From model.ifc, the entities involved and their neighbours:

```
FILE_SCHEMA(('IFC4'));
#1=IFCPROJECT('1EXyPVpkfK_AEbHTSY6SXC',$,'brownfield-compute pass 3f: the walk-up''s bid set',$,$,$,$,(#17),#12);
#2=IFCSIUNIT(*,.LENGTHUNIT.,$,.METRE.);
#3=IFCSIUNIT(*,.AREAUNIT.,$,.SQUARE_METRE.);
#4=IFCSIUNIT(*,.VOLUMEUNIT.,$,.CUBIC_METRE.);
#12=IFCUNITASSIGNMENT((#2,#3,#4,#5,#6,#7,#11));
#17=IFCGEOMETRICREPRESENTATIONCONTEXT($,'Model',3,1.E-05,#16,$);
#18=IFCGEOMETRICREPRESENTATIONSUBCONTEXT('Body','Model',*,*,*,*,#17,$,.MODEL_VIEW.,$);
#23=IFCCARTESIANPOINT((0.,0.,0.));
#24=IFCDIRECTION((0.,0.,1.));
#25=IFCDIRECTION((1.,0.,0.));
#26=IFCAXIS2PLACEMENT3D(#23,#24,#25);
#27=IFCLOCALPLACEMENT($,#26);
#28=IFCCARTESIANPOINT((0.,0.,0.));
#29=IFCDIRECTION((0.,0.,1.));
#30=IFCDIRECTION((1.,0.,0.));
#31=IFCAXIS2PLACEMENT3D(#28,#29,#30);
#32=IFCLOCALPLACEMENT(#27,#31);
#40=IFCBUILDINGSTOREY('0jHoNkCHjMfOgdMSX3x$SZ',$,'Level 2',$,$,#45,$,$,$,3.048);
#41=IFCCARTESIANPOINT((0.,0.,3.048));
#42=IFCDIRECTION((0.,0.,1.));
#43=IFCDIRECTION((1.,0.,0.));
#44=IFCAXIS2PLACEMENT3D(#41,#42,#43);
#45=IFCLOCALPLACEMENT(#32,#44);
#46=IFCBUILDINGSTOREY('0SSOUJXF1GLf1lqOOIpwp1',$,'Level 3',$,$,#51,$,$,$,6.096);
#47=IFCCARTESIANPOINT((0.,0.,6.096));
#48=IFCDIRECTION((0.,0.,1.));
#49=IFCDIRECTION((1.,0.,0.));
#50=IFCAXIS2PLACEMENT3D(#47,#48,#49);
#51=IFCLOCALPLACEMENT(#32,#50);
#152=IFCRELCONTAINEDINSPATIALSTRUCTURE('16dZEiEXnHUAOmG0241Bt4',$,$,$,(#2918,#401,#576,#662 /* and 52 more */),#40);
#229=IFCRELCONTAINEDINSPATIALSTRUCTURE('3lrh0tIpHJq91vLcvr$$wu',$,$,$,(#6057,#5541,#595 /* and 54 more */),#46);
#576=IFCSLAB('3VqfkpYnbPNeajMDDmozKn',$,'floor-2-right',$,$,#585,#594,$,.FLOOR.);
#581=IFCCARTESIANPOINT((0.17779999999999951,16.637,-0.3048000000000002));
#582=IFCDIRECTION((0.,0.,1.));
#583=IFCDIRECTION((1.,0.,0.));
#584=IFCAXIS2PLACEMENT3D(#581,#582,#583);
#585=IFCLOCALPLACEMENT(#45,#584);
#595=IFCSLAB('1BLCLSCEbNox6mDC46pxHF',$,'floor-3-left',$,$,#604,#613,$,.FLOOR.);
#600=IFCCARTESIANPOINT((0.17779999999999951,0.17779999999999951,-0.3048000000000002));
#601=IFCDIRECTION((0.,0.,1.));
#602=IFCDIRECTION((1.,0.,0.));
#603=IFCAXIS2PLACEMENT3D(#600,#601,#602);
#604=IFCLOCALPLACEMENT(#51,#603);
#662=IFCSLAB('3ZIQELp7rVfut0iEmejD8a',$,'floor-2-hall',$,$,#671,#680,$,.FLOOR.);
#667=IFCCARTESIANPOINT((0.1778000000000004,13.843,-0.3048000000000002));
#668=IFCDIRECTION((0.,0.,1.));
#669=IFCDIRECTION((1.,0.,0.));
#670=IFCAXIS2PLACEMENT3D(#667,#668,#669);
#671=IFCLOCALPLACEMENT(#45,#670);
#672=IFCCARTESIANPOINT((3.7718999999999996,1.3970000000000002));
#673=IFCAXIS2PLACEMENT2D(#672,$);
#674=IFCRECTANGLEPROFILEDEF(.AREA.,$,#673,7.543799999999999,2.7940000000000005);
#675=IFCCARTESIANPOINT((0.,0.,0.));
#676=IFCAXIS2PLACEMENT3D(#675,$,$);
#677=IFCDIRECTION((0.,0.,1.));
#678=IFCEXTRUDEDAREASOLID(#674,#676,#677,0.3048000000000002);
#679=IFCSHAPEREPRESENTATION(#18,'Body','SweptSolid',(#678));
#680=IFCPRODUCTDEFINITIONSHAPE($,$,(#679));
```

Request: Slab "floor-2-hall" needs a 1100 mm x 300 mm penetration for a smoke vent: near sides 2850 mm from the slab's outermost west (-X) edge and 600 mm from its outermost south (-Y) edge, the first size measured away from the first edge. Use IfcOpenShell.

```python
import numpy as np
import ifcopenshell
import ifcopenshell.api.feature
import ifcopenshell.api.geometry
import ifcopenshell.api.root
import ifcopenshell.geom
import ifcopenshell.util.placement
import ifcopenshell.util.representation
import ifcopenshell.util.shape
import ifcopenshell.util.unit

model = ifcopenshell.open("model.ifc")
unit_scale = ifcopenshell.util.unit.calculate_unit_scale(model)
settings = ifcopenshell.geom.settings()


def volume(element):
    """Net volume in cubic metres, openings subtracted."""
    shape = ifcopenshell.geom.create_shape(settings, element)
    return ifcopenshell.util.shape.get_volume(shape.geometry)


slab = model.by_id(662)
before = volume(slab)

# Extent in the slab's own axes, in metres. The edges named are its -X and -Y sides.
slab_shape = ifcopenshell.geom.create_shape(settings, slab)
vertices = ifcopenshell.util.shape.get_vertices(slab_shape.geometry)
x_min, y_min, bottom = vertices.min(axis=0)
top = vertices[:, 2].max()

opening = ifcopenshell.api.root.create_entity(model, ifc_class="IfcOpeningElement", name="Smoke vent opening", predefined_type="OPENING")
context = ifcopenshell.util.representation.get_context(model, "Model", "Body", "MODEL_VIEW")
width, depth = 1.1, 0.3
outline = [(0.0, 0.0), (width, 0.0), (width, depth), (0.0, depth), (0.0, 0.0)]
# Overshoot both faces by 50 mm so the cut is clean.
shape = ifcopenshell.api.geometry.add_slab_representation(
    model, context=context, depth=top - bottom + 0.1, polyline=outline
)
ifcopenshell.api.geometry.assign_representation(model, product=opening, representation=shape)

matrix = ifcopenshell.util.placement.get_local_placement(slab.ObjectPlacement)
matrix[:, 3] = matrix @ np.append(np.array([x_min + 2.85, y_min + 0.6, bottom - 0.05]) / unit_scale, 1.0)
ifcopenshell.api.geometry.edit_object_placement(model, product=opening, matrix=matrix, is_si=False)
ifcopenshell.api.feature.add_feature(model, feature=opening, element=slab)

after = volume(slab)

print(f"slab volume {before:.3f} -> {after:.3f} m3")

model.write("model_rev.ifc")
```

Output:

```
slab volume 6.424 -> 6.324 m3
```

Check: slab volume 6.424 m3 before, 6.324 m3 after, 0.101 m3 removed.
